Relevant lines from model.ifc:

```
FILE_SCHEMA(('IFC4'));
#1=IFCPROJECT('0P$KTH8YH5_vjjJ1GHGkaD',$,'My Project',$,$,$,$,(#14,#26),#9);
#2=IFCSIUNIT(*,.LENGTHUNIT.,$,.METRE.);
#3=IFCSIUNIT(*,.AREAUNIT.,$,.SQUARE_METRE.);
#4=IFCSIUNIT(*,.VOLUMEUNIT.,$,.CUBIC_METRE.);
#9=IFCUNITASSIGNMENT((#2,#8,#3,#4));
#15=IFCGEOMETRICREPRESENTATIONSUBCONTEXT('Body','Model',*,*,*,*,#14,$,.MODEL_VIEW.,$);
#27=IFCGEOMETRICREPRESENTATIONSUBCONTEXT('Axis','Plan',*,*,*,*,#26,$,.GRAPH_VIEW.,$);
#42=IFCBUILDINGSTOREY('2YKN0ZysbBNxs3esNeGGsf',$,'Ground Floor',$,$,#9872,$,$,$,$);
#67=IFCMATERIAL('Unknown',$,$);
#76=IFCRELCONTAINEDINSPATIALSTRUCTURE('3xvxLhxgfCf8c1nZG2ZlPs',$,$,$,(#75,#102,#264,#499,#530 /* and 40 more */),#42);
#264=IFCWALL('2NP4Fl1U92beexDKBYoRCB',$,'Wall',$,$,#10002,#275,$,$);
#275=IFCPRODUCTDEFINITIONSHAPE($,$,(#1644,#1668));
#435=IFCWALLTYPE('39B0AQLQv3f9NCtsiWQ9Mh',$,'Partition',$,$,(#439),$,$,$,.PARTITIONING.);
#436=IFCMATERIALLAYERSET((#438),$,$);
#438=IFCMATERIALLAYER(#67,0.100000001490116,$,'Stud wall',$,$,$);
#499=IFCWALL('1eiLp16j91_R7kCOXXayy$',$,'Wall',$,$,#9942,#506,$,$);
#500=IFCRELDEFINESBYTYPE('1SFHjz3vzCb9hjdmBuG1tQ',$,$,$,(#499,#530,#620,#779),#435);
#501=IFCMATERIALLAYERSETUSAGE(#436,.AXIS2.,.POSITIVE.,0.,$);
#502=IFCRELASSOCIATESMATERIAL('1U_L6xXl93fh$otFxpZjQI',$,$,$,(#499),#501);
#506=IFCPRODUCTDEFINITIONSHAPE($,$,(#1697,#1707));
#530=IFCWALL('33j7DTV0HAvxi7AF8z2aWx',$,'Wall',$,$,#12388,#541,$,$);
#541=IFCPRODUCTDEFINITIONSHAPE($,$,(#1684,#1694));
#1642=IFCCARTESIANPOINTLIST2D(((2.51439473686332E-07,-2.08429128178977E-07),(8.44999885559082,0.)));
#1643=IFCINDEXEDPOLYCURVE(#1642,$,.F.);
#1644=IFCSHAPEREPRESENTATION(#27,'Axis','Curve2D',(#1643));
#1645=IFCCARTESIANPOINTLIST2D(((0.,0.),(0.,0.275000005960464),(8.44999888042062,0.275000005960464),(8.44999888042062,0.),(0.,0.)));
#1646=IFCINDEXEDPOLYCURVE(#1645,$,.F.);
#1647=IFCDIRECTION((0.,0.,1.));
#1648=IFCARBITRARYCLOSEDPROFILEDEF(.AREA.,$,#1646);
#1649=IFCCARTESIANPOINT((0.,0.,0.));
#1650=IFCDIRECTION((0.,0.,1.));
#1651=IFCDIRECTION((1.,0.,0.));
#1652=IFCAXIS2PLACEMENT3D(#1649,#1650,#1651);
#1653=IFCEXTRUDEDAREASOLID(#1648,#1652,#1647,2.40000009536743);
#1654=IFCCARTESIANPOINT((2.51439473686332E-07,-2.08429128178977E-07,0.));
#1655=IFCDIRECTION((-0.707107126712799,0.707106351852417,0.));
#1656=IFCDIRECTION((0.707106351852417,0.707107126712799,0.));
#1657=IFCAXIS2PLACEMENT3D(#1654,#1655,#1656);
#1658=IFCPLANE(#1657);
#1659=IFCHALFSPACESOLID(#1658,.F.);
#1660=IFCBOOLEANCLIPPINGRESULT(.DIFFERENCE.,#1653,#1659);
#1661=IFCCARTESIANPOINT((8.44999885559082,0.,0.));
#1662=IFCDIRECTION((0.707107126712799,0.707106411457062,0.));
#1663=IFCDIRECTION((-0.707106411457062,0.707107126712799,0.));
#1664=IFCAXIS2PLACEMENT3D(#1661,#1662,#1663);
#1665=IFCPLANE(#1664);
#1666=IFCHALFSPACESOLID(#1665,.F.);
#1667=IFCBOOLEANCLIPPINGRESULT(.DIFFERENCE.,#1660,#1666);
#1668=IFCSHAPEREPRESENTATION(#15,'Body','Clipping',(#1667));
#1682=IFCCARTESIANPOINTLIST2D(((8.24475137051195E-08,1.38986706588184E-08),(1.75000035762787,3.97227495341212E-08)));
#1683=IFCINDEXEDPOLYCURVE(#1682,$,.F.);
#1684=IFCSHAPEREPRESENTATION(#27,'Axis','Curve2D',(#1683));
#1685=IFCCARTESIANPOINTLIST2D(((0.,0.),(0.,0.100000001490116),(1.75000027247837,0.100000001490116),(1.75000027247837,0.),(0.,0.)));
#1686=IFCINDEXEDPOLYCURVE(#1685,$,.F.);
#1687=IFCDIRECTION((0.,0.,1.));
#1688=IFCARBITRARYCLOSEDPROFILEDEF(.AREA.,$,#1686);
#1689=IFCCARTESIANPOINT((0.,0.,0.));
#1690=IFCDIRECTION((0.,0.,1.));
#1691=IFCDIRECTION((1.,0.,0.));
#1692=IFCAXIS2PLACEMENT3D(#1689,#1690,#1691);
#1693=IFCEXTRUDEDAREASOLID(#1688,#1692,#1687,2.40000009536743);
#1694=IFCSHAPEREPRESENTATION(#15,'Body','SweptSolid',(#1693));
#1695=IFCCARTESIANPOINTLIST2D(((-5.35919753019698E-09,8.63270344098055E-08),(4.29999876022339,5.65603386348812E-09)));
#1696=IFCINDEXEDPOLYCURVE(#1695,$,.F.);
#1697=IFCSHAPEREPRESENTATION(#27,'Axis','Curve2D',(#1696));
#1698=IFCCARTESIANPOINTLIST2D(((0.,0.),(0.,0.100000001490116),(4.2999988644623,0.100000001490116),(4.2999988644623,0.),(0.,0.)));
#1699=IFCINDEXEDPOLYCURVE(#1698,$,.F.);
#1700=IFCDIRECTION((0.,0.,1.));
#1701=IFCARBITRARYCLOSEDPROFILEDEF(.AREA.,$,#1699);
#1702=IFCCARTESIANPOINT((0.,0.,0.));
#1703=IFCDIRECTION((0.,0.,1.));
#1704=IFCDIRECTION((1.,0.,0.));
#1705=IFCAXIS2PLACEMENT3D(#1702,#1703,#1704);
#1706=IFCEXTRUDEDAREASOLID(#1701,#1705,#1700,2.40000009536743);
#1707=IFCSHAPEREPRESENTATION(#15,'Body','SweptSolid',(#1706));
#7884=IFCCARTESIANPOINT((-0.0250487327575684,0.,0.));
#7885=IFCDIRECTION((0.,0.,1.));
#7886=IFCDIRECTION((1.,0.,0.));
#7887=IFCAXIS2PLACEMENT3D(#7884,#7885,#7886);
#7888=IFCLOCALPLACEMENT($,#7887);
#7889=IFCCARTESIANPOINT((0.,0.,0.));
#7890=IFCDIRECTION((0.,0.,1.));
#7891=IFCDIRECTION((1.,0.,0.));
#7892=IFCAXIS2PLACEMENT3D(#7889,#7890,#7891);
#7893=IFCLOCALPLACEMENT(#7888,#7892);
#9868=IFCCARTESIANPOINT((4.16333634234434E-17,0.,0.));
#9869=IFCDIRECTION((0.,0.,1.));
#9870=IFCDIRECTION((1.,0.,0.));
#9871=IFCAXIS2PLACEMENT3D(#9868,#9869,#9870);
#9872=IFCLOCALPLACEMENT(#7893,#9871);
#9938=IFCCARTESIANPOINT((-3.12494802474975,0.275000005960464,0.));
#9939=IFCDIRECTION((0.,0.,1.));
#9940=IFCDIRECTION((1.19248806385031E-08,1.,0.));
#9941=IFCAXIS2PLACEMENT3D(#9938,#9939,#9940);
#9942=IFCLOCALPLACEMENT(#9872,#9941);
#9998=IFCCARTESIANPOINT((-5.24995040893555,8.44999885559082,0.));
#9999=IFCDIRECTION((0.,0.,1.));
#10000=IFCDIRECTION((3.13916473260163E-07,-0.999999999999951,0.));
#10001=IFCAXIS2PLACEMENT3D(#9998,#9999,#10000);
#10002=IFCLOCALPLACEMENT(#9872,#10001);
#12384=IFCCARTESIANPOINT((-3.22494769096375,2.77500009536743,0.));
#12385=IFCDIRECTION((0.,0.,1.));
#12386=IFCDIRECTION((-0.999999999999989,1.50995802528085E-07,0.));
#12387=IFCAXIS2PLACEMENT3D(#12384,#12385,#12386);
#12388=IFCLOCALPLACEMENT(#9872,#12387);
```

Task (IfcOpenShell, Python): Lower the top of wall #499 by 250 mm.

```python
import ifcopenshell
import ifcopenshell.geom
import ifcopenshell.util.representation
import ifcopenshell.util.shape

model = ifcopenshell.open("model.ifc")
settings = ifcopenshell.geom.settings()


def volume(element):
    """Net volume in cubic metres, openings subtracted."""
    shape = ifcopenshell.geom.create_shape(settings, element)
    return ifcopenshell.util.shape.get_volume(shape.geometry)


wall = model.by_id(499)
before = volume(wall)

body = ifcopenshell.util.representation.get_representation(wall, "Model", "Body")
solid = body.Items[0]
old_height = solid.Depth
solid.Depth -= 0.25
after = volume(wall)

print(f"height {old_height:g} -> {solid.Depth:g}, volume {before:.3f} -> {after:.3f} m3")

model.write("model_rev.ifc")
```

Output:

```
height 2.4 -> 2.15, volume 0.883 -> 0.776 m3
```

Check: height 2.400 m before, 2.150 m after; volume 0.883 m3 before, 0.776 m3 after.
